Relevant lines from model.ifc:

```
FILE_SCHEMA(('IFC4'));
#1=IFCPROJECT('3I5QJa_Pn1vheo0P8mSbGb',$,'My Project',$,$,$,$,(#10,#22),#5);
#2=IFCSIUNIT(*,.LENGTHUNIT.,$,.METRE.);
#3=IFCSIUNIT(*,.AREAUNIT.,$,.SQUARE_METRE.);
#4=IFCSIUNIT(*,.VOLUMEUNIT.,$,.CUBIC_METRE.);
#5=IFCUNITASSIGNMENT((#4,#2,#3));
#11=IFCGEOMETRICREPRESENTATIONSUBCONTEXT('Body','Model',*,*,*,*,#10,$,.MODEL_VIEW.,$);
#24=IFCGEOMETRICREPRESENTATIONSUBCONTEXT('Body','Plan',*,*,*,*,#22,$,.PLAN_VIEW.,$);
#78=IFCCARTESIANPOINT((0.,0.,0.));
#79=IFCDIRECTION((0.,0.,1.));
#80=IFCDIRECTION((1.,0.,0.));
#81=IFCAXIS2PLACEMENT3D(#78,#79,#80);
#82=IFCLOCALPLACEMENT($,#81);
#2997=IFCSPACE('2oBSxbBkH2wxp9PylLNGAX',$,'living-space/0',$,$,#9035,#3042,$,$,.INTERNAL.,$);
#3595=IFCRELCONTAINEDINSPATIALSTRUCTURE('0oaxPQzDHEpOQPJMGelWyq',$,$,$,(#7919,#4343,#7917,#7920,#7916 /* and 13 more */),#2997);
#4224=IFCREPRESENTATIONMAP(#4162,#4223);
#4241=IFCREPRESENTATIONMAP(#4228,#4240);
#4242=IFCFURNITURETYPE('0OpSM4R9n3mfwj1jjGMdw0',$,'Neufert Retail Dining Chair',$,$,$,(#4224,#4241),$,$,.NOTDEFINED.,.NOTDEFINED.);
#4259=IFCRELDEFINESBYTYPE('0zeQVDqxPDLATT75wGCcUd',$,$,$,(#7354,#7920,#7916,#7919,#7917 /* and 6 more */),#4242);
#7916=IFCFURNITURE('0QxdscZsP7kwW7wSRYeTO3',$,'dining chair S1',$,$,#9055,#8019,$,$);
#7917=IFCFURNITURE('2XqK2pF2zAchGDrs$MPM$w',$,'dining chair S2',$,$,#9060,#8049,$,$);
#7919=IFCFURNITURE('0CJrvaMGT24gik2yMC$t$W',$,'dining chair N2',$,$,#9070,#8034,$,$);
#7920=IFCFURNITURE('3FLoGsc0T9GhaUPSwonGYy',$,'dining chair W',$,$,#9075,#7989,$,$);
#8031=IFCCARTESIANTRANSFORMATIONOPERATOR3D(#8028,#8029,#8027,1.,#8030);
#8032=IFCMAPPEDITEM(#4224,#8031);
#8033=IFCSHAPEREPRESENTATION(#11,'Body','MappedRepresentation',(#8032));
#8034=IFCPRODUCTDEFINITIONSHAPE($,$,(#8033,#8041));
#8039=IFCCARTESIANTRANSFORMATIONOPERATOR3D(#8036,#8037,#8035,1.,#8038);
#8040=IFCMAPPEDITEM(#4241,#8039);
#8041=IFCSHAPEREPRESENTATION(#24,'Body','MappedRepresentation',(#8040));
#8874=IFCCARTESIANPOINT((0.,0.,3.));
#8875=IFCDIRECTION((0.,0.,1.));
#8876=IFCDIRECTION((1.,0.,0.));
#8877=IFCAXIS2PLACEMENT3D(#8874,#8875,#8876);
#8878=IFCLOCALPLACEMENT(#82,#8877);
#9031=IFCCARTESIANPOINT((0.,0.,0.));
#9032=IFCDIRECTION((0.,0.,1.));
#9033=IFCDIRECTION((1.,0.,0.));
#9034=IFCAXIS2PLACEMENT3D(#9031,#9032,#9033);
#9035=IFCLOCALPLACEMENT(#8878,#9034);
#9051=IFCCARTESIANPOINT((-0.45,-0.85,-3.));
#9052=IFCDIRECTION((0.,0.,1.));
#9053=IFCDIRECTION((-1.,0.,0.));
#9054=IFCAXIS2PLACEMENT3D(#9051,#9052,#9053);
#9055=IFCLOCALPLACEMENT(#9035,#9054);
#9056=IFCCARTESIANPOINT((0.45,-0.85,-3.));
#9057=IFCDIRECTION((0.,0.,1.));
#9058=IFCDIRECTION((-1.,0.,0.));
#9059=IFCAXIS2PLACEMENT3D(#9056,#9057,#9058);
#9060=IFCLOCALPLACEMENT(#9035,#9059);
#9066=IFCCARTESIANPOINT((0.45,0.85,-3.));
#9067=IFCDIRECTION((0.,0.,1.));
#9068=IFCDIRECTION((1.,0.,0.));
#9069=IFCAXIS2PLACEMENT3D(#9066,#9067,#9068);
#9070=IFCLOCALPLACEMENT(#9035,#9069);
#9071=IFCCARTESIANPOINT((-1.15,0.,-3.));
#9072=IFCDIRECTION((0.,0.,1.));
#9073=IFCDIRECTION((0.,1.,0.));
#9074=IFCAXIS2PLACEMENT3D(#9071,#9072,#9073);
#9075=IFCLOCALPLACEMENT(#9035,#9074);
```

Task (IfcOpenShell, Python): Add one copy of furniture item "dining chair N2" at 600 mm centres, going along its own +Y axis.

```python
import ifcopenshell
import ifcopenshell.api.geometry
import ifcopenshell.api.root
import ifcopenshell.util.element
import ifcopenshell.util.placement

model = ifcopenshell.open("model.ifc")

source = model.by_id(7919)
base = ifcopenshell.util.placement.get_local_placement(source.ObjectPlacement)
step = base[:3, 1] * 0.6

for i in range(1, 2):
    copy = ifcopenshell.api.root.copy_class(model, product=source)
    copy.Representation = ifcopenshell.util.element.copy_deep(
        model, source.Representation, exclude=["IfcGeometricRepresentationContext", "IfcRepresentationMap"]
    )
    matrix = base.copy()
    matrix[:3, 3] += i * step
    print("added at", matrix[:3, 3].round(3) + 0.0)
    ifcopenshell.api.geometry.edit_object_placement(model, product=copy, matrix=matrix, is_si=False)

model.write("model_rev.ifc")
```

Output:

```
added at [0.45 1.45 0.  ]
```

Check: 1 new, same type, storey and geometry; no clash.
